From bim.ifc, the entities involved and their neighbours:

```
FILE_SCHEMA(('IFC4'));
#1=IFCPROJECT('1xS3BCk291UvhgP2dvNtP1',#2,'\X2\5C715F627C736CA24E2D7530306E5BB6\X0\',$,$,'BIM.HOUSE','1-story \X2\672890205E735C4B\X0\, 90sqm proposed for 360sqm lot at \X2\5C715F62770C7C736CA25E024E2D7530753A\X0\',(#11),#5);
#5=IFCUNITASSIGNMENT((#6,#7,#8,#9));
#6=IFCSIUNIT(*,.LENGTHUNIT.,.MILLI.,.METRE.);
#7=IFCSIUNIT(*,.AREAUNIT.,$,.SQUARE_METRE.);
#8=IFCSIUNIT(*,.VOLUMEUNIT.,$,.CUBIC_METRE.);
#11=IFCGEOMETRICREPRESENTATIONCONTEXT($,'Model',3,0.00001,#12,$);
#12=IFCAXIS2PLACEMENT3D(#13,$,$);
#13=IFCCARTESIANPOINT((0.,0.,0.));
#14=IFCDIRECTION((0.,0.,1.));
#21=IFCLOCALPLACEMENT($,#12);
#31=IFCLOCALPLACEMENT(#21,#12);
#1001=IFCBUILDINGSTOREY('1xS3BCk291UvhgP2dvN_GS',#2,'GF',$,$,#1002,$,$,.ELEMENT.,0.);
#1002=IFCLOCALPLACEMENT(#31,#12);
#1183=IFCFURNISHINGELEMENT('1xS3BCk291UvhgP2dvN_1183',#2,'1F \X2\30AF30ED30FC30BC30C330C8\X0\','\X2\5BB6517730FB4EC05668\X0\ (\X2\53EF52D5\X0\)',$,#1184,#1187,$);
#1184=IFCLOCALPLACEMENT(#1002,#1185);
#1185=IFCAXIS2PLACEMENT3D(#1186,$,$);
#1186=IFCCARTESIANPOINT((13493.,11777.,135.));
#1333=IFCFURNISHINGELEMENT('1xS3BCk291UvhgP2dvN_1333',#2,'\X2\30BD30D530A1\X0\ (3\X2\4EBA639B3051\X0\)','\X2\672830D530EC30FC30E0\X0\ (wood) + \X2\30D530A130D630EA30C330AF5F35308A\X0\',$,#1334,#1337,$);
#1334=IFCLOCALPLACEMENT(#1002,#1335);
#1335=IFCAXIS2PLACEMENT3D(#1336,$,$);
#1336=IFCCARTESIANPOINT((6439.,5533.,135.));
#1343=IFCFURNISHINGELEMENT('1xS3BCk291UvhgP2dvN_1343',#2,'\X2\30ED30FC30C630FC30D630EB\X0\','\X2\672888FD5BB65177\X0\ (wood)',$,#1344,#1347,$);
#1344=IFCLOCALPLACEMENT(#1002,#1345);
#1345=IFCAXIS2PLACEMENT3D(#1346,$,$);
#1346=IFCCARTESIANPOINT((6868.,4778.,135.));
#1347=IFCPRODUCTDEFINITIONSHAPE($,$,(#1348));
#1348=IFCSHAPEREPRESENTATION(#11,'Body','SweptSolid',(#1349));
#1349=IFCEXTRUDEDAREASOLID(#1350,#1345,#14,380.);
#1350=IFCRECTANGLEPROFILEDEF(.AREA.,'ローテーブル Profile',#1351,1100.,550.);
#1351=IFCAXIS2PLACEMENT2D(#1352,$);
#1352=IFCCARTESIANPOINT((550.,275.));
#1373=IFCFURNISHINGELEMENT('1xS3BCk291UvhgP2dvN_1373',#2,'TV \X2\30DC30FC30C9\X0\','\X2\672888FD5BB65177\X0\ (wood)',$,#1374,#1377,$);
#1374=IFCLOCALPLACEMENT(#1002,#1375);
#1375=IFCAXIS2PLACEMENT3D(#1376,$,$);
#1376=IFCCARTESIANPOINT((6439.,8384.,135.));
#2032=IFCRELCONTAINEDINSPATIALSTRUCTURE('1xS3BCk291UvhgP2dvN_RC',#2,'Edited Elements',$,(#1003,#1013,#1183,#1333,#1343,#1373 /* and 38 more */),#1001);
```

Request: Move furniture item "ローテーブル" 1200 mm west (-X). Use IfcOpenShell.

```python
import ifcopenshell
import ifcopenshell.api.geometry
import ifcopenshell.util.placement
import ifcopenshell.util.unit

model = ifcopenshell.open("bim.ifc")
unit_scale = ifcopenshell.util.unit.calculate_unit_scale(model)

item = model.by_id(1343)
matrix = ifcopenshell.util.placement.get_local_placement(item.ObjectPlacement)
matrix[0, 3] -= 1.2 / unit_scale
ifcopenshell.api.geometry.edit_object_placement(model, product=item, matrix=matrix, is_si=False)

print(ifcopenshell.util.placement.get_local_placement(item.ObjectPlacement).round(3) + 0.0)

model.write("bim_rev.ifc")
```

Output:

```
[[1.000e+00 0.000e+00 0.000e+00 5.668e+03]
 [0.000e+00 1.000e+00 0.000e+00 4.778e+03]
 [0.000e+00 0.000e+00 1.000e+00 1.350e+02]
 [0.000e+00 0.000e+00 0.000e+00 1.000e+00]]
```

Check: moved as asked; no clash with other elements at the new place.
